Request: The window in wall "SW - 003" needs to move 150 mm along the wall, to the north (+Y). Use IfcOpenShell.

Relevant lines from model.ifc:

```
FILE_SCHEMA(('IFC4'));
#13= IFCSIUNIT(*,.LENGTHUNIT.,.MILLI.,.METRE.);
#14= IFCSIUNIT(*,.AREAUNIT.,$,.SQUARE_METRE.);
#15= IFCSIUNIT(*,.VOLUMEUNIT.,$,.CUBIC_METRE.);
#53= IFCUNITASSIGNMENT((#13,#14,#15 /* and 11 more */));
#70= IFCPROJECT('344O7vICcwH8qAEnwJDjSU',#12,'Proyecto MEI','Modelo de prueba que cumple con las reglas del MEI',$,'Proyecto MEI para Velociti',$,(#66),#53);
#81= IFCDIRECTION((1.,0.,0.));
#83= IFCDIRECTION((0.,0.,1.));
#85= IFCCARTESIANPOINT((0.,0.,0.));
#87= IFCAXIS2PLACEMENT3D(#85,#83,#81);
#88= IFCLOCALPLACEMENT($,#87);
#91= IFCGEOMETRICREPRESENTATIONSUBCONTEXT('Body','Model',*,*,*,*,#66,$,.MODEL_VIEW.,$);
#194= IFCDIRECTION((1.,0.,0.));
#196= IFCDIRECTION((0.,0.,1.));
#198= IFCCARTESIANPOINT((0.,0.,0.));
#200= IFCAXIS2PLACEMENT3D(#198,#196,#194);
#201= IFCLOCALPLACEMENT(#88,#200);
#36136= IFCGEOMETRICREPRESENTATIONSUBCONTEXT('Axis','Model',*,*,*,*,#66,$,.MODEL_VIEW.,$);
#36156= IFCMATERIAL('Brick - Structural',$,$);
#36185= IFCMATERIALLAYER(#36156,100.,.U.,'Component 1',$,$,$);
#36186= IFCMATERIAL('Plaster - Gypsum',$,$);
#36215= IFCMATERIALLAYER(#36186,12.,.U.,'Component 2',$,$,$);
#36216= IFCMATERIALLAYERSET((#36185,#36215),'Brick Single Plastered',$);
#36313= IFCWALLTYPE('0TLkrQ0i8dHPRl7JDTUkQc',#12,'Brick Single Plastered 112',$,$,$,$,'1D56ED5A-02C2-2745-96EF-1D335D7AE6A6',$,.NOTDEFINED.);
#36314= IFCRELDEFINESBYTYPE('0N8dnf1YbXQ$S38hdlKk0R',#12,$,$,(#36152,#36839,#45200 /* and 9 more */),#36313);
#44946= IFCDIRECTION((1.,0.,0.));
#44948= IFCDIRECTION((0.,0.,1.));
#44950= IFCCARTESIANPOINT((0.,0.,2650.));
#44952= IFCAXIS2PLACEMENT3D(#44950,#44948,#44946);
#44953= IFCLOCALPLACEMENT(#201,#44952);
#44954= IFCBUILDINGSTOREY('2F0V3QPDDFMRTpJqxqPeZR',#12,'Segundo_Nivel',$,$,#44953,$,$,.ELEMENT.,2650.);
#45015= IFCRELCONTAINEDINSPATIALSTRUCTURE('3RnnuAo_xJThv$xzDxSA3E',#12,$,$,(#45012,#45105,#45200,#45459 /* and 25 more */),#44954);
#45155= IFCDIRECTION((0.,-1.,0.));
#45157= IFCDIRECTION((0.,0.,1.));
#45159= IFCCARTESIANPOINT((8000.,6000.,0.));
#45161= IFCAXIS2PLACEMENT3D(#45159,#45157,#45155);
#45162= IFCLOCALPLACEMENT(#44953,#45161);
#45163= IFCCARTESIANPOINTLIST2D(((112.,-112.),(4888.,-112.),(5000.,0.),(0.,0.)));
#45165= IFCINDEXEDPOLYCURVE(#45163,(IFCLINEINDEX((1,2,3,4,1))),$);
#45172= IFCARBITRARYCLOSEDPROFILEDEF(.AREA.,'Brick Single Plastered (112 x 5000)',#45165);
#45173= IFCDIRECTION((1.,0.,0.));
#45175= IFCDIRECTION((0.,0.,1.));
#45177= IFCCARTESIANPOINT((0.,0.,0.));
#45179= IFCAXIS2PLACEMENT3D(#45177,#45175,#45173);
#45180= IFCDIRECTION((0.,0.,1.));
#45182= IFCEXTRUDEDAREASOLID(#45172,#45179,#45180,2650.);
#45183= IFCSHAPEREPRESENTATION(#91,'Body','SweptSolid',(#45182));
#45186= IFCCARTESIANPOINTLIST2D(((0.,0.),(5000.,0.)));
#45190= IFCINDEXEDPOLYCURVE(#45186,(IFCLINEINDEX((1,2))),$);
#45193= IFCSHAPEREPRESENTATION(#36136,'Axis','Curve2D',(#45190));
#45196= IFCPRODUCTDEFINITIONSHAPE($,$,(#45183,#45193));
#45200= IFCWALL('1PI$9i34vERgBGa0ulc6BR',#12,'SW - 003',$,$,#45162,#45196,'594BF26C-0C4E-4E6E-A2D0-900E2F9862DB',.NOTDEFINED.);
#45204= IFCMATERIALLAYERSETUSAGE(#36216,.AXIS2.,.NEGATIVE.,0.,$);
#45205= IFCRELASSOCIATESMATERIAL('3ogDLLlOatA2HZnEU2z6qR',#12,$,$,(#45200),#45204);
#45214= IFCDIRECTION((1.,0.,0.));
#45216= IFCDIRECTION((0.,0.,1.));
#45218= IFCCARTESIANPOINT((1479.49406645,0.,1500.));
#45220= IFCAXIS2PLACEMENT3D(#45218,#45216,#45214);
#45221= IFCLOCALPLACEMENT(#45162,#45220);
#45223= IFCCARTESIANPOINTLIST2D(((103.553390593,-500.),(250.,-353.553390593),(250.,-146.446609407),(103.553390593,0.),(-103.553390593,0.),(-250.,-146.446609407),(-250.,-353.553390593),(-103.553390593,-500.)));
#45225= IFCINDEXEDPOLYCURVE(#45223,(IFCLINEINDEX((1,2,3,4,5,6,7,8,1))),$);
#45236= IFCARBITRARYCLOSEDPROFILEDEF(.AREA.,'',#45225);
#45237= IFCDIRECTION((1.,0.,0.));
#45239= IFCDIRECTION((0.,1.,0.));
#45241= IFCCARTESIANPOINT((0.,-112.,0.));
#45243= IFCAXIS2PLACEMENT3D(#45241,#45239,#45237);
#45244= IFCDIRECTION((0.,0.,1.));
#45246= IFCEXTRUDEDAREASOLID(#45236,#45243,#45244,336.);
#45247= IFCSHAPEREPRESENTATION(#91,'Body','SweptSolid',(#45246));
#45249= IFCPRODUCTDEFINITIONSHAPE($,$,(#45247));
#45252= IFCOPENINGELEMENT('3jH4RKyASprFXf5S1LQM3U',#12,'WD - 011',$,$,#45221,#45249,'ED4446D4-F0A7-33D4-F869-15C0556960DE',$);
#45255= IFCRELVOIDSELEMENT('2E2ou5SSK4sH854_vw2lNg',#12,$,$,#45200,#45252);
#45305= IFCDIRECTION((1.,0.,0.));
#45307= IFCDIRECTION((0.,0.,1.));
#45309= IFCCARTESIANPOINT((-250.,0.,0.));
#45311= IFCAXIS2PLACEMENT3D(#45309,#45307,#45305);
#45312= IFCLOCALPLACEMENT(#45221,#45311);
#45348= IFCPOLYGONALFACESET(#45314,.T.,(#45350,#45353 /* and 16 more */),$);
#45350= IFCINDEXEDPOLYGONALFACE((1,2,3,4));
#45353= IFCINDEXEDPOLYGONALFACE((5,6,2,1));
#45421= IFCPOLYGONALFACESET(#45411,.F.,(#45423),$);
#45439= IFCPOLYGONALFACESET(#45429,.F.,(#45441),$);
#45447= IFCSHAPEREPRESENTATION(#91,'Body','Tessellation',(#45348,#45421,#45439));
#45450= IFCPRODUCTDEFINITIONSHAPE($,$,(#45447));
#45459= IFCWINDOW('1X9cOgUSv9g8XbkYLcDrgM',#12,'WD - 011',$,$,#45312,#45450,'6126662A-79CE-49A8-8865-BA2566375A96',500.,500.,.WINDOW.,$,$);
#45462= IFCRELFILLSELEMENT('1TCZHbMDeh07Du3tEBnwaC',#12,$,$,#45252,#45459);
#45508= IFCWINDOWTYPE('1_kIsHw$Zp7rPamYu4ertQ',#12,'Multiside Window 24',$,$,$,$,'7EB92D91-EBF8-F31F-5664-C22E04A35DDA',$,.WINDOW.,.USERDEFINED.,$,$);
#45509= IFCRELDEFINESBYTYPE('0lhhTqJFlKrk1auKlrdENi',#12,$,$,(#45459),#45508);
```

```python
import ifcopenshell
import ifcopenshell.api.geometry
import ifcopenshell.util.placement
import ifcopenshell.util.unit

model = ifcopenshell.open("model.ifc")
unit_scale = ifcopenshell.util.unit.calculate_unit_scale(model)

window = model.by_guid("1X9cOgUSv9g8XbkYLcDrgM")
opening = window.FillsVoids[0].RelatingOpeningElement
wall = opening.VoidsElements[0].RelatingBuildingElement

wall_matrix = ifcopenshell.util.placement.get_local_placement(wall.ObjectPlacement)
shift = wall_matrix[:3, 0] * -0.15 / unit_scale
before = ifcopenshell.util.placement.get_local_placement(window.ObjectPlacement)[:3, 3].copy()

# The window is placed relative to its opening, so it follows when the opening moves.
matrix = ifcopenshell.util.placement.get_local_placement(opening.ObjectPlacement)
matrix[:3, 3] += shift
ifcopenshell.api.geometry.edit_object_placement(
    model, product=opening, matrix=matrix, is_si=False, should_transform_children=True
)

after = ifcopenshell.util.placement.get_local_placement(window.ObjectPlacement)[:3, 3]
print("window moved by", (after - before).round(3) + 0.0)

model.write("model_updated.ifc")
```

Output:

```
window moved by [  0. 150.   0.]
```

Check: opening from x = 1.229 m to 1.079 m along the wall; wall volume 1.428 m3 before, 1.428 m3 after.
